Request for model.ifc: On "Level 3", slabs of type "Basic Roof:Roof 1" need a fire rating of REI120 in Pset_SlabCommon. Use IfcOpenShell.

First a look at what the model holds.

```python
import ifcopenshell
import ifcopenshell.util.element

model = ifcopenshell.open("model.ifc")
print(model.schema)
storey = next(s for s in model.by_type("IfcBuildingStorey") if s.Name == "Level 3")
slabs = [e for e in ifcopenshell.util.element.get_decomposition(storey) if e.is_a("IfcSlab")]
seen = {}
for e in slabs:
    element_type = ifcopenshell.util.element.get_type(e)
    key = (element_type.Name if element_type != e and element_type else None, ifcopenshell.util.element.get_pset(e, "Pset_SlabCommon", "FireRating"))
    seen[key] = seen.get(key, 0) + 1
for (name, value), count in sorted(seen.items(), key=str):
    print(count, "x", name, "|", value)
```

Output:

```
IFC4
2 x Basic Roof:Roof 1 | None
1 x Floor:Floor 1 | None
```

```python
import ifcopenshell
import ifcopenshell.api.pset
import ifcopenshell.util.element

model = ifcopenshell.open("model.ifc")

storey = next(s for s in model.by_type("IfcBuildingStorey") if s.Name == "Level 3")
slabs = [e for e in ifcopenshell.util.element.get_decomposition(storey) if e.is_a("IfcSlab")]

count = 0
for e in slabs:
    element_type = ifcopenshell.util.element.get_type(e)
    if element_type in (None, e) or element_type.Name != "Basic Roof:Roof 1":
        continue
    # add_pset returns the element's existing set when there is one.
    pset = ifcopenshell.api.pset.add_pset(model, product=e, name="Pset_SlabCommon")
    ifcopenshell.api.pset.edit_pset(model, pset=pset, properties={"FireRating": "REI120"})
    count += 1

print(count, "slabs updated")

model.write("model-out.ifc")
```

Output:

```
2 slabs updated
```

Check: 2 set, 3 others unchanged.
